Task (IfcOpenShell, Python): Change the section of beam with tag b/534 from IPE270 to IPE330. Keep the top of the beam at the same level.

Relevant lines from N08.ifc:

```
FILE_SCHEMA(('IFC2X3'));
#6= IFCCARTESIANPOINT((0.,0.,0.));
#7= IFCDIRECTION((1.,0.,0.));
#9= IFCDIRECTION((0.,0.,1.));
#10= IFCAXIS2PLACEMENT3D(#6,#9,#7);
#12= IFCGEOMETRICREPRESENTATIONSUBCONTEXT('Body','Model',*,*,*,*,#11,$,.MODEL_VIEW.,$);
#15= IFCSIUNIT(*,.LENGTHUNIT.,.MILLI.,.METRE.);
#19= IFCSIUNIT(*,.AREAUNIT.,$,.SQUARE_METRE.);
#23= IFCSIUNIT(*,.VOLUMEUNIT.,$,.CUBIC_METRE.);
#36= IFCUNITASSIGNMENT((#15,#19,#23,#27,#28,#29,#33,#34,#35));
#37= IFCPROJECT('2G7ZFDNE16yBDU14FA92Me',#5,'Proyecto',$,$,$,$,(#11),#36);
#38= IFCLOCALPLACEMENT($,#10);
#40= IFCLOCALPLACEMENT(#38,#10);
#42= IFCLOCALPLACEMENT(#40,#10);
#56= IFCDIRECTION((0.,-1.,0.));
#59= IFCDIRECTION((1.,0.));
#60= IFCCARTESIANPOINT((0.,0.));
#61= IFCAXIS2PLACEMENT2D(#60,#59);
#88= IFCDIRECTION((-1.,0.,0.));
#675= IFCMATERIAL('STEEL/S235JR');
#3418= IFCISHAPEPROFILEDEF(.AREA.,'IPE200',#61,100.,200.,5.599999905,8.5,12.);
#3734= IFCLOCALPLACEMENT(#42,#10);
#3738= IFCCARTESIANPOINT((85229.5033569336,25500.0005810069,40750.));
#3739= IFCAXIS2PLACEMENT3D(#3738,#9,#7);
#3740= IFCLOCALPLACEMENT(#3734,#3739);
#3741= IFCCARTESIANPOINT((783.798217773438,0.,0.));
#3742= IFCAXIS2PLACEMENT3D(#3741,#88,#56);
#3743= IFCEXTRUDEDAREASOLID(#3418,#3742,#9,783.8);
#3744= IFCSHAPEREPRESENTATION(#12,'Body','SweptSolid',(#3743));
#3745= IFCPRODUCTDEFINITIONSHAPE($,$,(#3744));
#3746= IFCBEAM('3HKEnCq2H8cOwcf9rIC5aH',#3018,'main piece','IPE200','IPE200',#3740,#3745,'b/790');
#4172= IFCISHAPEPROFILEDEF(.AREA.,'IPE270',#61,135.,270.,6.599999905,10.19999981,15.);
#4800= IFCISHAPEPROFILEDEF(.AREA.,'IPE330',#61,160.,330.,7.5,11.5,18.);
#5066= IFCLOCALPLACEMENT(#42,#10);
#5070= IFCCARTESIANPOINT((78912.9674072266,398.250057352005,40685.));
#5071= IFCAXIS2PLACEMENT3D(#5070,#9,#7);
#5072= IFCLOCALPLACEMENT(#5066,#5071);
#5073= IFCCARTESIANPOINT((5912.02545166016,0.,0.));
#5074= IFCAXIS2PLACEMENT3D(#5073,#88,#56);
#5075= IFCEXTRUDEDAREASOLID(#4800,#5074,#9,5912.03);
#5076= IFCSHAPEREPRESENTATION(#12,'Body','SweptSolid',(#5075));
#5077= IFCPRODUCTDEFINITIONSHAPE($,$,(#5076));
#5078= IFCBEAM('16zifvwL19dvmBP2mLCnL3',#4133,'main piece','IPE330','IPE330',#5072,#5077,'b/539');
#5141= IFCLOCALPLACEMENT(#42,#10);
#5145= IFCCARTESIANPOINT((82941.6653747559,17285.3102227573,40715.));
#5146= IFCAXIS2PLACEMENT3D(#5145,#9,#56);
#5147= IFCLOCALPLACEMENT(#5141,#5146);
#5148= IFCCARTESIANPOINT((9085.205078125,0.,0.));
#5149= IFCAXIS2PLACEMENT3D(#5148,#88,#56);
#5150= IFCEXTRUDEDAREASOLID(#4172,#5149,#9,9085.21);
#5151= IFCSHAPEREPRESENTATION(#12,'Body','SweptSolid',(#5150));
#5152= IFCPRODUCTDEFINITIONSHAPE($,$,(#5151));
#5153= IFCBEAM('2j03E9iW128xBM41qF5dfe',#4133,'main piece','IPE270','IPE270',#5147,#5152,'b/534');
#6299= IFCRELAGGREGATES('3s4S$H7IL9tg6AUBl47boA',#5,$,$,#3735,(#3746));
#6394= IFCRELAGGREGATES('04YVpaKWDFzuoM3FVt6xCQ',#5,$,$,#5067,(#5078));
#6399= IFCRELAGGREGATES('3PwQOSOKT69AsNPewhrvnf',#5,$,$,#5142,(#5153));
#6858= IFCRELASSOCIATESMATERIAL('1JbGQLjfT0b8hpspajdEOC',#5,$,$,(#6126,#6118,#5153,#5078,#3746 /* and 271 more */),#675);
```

```python
import ifcopenshell
import ifcopenshell.util.element
import ifcopenshell.util.representation

model = ifcopenshell.open("N08.ifc")

member = model.by_guid("2j03E9iW128xBM41qF5dfe")
source = next(p for p in model.by_type("IfcIShapeProfileDef") if p.ProfileName == "IPE330")

body = ifcopenshell.util.representation.get_representation(member, "Model", "Body")
solid = body.Items[0]
old_profile = solid.SweptArea

# Copy the section's sizes but keep this member's own profile position.
profile = ifcopenshell.util.element.copy(model, source)
# Profiles are centred, so shift by half the change in depth to hold the top.
shift = (old_profile.OverallDepth - profile.OverallDepth) / 2
x, y = old_profile.Position.Location.Coordinates
up = (0.0, 1.0)  # upwards, in the solid's own plane
location = model.createIfcCartesianPoint((x + up[0] * shift, y + up[1] * shift))
profile.Position = model.createIfcAxis2Placement2D(location, old_profile.Position.RefDirection)
solid.SweptArea = profile
if not model.get_total_inverses(old_profile):
    ifcopenshell.util.element.remove_deep2(model, old_profile)
member.Description = member.Description.replace("IPE270", "IPE330")
member.ObjectType = member.ObjectType.replace("IPE270", "IPE330")

print(solid.SweptArea)

model.write("N08_v2.ifc")
```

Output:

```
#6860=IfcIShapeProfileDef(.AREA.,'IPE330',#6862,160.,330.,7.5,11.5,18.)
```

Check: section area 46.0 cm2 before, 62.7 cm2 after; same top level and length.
